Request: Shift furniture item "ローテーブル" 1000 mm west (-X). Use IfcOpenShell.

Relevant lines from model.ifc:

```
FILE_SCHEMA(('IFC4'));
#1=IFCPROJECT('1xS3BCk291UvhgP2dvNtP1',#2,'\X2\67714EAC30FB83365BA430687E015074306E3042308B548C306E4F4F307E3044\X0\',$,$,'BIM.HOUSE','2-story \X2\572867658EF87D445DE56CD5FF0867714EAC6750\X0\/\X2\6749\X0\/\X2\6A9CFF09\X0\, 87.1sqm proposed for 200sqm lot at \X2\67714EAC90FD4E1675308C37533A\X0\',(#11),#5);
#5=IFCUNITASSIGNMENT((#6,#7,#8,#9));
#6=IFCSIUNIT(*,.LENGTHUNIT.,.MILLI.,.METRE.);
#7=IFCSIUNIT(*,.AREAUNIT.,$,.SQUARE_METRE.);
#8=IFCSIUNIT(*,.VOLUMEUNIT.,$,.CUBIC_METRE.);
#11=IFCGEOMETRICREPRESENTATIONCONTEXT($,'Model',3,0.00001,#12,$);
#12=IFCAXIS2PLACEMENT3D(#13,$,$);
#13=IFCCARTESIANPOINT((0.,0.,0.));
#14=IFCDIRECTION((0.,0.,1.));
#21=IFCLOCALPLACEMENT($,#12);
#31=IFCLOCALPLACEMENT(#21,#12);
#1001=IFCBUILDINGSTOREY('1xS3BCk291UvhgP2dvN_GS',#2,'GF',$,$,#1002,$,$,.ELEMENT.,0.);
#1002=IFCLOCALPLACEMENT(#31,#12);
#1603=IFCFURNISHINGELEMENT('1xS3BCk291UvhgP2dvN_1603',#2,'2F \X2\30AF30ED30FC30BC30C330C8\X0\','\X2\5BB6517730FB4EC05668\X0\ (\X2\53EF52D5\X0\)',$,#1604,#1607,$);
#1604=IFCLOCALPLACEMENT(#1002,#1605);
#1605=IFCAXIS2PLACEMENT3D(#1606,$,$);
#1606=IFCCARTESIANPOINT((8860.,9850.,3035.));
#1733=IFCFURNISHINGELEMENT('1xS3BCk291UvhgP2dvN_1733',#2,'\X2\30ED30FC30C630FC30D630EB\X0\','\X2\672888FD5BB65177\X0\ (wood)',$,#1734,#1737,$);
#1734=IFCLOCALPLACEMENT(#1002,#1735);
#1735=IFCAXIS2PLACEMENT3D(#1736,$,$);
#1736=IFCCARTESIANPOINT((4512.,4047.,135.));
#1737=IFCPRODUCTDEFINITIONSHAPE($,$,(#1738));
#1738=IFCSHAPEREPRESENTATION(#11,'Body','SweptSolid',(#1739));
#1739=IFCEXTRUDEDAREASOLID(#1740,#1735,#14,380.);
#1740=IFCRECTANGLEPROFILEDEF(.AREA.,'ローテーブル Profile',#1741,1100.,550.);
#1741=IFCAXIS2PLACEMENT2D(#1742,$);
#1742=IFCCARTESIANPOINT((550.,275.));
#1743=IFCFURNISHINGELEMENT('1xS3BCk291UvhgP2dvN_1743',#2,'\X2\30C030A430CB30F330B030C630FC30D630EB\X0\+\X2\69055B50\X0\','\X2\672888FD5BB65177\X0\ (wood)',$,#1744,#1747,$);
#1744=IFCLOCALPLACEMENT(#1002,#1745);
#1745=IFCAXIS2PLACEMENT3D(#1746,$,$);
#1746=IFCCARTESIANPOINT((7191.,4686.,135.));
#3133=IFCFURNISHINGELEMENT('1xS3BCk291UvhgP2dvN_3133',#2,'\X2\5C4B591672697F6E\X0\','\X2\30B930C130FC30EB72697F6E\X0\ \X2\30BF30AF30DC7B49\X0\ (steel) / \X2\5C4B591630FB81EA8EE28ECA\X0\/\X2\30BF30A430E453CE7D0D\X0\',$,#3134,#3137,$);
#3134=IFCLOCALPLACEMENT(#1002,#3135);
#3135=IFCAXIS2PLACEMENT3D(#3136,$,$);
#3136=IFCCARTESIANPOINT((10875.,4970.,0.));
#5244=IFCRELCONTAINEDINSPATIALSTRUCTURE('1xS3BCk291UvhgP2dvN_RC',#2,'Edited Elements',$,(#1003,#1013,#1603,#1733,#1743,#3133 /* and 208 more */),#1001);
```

```python
import ifcopenshell
import ifcopenshell.api.geometry
import ifcopenshell.util.placement
import ifcopenshell.util.unit

model = ifcopenshell.open("model.ifc")
unit_scale = ifcopenshell.util.unit.calculate_unit_scale(model)

item = model.by_guid("1xS3BCk291UvhgP2dvN_1733")
matrix = ifcopenshell.util.placement.get_local_placement(item.ObjectPlacement)
matrix[0, 3] -= 1 / unit_scale
ifcopenshell.api.geometry.edit_object_placement(model, product=item, matrix=matrix, is_si=False)

print(ifcopenshell.util.placement.get_local_placement(item.ObjectPlacement).round(3) + 0.0)

model.write("model-out.ifc")
```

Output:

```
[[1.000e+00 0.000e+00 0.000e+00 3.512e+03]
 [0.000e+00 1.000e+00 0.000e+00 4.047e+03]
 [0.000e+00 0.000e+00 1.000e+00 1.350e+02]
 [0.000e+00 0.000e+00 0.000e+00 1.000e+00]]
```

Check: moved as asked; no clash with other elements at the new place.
